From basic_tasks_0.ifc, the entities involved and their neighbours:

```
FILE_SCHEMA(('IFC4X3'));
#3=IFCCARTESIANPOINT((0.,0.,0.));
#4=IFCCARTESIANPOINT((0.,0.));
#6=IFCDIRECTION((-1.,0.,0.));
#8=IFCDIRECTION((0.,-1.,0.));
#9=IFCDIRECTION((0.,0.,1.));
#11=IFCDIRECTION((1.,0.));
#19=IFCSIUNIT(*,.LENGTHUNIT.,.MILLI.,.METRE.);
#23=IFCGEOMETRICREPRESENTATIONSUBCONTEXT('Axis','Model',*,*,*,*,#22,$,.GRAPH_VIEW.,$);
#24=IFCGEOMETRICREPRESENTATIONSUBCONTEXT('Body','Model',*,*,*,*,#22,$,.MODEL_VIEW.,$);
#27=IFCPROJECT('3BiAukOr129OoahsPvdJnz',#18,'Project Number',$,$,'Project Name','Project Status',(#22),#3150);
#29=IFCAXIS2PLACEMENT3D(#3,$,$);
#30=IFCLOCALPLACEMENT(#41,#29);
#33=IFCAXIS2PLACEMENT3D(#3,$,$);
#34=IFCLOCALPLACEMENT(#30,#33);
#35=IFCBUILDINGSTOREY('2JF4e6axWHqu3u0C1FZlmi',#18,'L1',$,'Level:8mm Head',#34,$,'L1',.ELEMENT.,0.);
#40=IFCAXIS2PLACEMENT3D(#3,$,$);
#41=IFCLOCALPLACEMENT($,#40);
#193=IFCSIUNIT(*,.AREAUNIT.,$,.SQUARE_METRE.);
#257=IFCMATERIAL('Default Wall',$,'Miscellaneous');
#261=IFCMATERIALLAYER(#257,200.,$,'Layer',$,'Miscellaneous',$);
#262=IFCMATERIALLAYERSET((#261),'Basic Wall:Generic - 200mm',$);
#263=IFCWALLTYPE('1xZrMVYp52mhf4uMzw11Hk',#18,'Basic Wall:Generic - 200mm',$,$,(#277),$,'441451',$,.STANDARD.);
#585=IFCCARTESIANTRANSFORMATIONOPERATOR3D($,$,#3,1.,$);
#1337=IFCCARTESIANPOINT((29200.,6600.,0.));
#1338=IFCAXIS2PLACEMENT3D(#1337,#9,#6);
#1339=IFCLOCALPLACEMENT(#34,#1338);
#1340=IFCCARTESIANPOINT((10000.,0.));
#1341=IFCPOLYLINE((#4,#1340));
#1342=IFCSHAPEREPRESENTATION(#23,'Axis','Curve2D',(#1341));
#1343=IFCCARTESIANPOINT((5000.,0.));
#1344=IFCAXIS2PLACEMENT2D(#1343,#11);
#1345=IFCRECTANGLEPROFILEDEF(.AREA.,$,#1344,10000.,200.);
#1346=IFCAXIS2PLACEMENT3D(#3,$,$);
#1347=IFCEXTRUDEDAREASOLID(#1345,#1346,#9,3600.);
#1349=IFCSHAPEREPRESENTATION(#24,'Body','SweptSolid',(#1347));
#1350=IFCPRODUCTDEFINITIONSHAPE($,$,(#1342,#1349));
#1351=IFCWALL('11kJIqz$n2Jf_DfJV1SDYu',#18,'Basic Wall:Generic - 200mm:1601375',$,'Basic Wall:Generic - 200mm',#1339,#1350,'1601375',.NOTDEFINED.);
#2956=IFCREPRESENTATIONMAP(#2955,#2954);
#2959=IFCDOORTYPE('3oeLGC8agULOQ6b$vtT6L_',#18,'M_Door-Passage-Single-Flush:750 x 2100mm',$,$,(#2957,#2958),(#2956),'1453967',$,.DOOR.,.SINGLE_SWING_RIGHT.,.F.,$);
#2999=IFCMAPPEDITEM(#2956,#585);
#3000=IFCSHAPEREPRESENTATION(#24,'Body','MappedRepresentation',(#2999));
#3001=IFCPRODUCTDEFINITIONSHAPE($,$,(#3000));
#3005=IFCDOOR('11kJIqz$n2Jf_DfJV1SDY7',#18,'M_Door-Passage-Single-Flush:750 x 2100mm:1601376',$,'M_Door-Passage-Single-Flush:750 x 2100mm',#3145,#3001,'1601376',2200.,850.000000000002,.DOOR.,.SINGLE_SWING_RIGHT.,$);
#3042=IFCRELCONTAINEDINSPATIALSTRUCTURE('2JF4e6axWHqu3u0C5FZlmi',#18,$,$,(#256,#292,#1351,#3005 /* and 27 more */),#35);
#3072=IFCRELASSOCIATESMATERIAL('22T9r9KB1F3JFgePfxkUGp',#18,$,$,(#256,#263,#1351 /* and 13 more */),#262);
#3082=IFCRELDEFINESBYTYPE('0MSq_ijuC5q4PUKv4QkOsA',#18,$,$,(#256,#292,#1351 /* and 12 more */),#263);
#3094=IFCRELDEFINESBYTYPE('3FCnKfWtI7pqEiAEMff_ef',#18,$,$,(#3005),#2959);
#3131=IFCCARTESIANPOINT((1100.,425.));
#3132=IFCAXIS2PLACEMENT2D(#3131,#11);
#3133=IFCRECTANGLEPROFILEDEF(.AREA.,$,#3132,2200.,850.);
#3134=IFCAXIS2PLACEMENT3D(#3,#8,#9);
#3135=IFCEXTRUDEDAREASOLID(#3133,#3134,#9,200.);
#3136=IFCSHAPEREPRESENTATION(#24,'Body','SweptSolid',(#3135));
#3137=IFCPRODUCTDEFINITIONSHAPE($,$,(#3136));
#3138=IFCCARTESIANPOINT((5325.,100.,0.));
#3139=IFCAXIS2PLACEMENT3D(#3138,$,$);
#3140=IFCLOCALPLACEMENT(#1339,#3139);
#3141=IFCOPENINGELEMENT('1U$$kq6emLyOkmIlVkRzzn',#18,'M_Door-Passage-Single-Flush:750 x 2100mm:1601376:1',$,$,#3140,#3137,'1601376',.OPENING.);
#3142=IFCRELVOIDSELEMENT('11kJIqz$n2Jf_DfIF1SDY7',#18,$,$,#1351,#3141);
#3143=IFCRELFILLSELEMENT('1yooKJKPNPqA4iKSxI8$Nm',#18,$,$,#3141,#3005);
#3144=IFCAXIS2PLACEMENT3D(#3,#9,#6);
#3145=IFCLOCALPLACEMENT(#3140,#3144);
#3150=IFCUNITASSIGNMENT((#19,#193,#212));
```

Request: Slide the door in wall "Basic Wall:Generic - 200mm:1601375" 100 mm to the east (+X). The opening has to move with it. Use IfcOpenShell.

```python
import ifcopenshell
import ifcopenshell.api.geometry
import ifcopenshell.util.placement

model = ifcopenshell.open("basic_tasks_0.ifc")

door = model.by_id(3005)
opening = door.FillsVoids[0].RelatingOpeningElement
wall = opening.VoidsElements[0].RelatingBuildingElement

wall_matrix = ifcopenshell.util.placement.get_local_placement(wall.ObjectPlacement)
shift = wall_matrix[:3, 0] * -100.0
before = ifcopenshell.util.placement.get_local_placement(door.ObjectPlacement)[:3, 3].copy()

# The door is placed relative to its opening, so it follows when the opening moves.
matrix = ifcopenshell.util.placement.get_local_placement(opening.ObjectPlacement)
matrix[:3, 3] += shift
ifcopenshell.api.geometry.edit_object_placement(
    model, product=opening, matrix=matrix, is_si=False, should_transform_children=True
)

after = ifcopenshell.util.placement.get_local_placement(door.ObjectPlacement)[:3, 3]
print("door moved by", (after - before).round(3) + 0.0)

model.write("basic_tasks_0_v2.ifc")
```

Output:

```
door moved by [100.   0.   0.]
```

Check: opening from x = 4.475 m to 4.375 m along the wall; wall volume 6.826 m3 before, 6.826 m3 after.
